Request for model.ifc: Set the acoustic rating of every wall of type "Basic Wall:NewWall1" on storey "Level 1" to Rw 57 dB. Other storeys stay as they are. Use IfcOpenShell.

First a look at what the model holds.

```python
import ifcopenshell
import ifcopenshell.util.element

model = ifcopenshell.open("model.ifc")
print(model.schema)
storey = next(s for s in model.by_type("IfcBuildingStorey") if s.Name == "Level 1")
walls = [e for e in ifcopenshell.util.element.get_decomposition(storey) if e.is_a("IfcWall")]
seen = {}
for e in walls:
    element_type = ifcopenshell.util.element.get_type(e)
    key = (element_type.Name if element_type != e and element_type else None, ifcopenshell.util.element.get_pset(e, "Pset_WallCommon", "AcousticRating"))
    seen[key] = seen.get(key, 0) + 1
for (name, value), count in sorted(seen.items(), key=str):
    print(count, "x", name, "|", value)
```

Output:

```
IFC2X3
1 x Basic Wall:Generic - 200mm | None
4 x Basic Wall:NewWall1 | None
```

```python
import ifcopenshell
import ifcopenshell.api.pset
import ifcopenshell.util.element

model = ifcopenshell.open("model.ifc")

storey = next(s for s in model.by_type("IfcBuildingStorey") if s.Name == "Level 1")
walls = [e for e in ifcopenshell.util.element.get_decomposition(storey) if e.is_a("IfcWall")]

count = 0
for e in walls:
    element_type = ifcopenshell.util.element.get_type(e)
    if element_type in (None, e) or element_type.Name != "Basic Wall:NewWall1":
        continue
    # add_pset returns the element's existing set when there is one.
    pset = ifcopenshell.api.pset.add_pset(model, product=e, name="Pset_WallCommon")
    ifcopenshell.api.pset.edit_pset(model, pset=pset, properties={"AcousticRating": "Rw 57 dB"})
    count += 1

print(count, "walls updated")

model.write("model-out.ifc")
```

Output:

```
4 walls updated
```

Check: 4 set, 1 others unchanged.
